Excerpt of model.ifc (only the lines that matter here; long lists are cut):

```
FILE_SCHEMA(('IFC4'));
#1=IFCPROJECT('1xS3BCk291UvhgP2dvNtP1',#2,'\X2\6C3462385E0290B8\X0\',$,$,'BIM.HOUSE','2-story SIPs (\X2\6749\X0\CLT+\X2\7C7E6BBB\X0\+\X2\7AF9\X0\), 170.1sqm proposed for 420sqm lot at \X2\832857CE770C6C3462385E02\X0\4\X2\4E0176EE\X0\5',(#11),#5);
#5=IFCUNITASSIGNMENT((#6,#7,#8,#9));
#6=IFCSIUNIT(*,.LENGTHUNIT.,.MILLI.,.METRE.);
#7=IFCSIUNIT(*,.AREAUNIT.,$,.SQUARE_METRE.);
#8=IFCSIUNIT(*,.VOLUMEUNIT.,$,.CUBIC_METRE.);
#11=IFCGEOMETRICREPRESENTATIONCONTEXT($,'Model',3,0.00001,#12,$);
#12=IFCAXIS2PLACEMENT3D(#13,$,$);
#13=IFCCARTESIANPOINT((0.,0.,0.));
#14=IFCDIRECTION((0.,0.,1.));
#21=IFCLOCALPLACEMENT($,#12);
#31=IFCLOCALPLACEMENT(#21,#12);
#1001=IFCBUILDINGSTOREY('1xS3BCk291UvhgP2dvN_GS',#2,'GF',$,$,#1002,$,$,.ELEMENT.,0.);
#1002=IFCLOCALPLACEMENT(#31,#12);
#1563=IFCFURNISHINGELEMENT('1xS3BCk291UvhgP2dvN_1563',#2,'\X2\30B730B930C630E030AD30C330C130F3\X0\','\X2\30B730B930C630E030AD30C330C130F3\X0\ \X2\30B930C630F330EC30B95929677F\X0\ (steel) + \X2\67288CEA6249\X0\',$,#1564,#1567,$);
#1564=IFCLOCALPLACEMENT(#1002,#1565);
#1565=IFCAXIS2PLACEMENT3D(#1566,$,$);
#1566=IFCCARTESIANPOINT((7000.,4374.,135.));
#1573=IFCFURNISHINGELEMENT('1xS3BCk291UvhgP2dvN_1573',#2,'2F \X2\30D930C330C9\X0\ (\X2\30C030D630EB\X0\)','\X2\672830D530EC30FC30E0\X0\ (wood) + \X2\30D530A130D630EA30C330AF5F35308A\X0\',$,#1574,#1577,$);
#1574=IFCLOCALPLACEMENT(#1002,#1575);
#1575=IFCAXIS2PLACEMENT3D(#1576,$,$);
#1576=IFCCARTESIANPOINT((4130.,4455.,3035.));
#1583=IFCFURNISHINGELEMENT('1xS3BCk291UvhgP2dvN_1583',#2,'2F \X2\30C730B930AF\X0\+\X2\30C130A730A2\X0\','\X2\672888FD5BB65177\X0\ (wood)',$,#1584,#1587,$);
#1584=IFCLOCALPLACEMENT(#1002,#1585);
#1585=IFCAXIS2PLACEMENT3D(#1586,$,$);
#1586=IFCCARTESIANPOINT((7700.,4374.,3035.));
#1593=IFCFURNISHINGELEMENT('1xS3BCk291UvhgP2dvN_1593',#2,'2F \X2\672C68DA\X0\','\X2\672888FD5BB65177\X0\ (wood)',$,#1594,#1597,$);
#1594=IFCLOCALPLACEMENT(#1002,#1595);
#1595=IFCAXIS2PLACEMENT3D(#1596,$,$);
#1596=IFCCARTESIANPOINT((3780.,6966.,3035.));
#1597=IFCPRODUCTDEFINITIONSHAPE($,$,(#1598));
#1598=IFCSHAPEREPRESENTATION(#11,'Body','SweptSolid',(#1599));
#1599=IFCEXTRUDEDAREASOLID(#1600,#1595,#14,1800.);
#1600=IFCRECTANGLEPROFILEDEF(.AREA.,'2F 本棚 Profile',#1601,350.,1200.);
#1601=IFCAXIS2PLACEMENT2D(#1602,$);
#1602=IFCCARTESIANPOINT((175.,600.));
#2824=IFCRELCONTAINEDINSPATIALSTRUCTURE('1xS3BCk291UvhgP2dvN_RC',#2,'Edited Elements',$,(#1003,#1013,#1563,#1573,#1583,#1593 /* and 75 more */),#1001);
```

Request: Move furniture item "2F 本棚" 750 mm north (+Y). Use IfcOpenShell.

```python
import ifcopenshell
import ifcopenshell.api.geometry
import ifcopenshell.util.placement
import ifcopenshell.util.unit

model = ifcopenshell.open("model.ifc")
unit_scale = ifcopenshell.util.unit.calculate_unit_scale(model)

item = model.by_guid("1xS3BCk291UvhgP2dvN_1593")
matrix = ifcopenshell.util.placement.get_local_placement(item.ObjectPlacement)
matrix[1, 3] += 0.75 / unit_scale
ifcopenshell.api.geometry.edit_object_placement(model, product=item, matrix=matrix, is_si=False)

print(ifcopenshell.util.placement.get_local_placement(item.ObjectPlacement).round(3) + 0.0)

model.write("model_v2.ifc")
```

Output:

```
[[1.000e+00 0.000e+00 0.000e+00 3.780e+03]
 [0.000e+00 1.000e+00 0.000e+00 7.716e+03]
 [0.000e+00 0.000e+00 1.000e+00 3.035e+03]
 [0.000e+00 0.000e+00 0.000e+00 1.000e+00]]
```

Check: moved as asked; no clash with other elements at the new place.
